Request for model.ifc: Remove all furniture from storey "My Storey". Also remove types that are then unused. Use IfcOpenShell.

First a look at what the model holds.

```python
import ifcopenshell
import ifcopenshell.util.element

model = ifcopenshell.open("model.ifc")
print(model.schema)
storey = next(s for s in model.by_type("IfcBuildingStorey") if s.Name == "My Storey")
furniture = [e for e in ifcopenshell.util.element.get_decomposition(storey) if e.is_a("IfcFurnishingElement")]
seen = {}
for e in furniture:
    element_type = ifcopenshell.util.element.get_type(e)
    name = element_type.Name if element_type not in (None, e) else None
    seen[name] = seen.get(name, 0) + 1
for name, count in sorted(seen.items(), key=str):
    print(count, "x", name)
```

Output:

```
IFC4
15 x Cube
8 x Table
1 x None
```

```python
import ifcopenshell
import ifcopenshell.api.root
import ifcopenshell.util.element

model = ifcopenshell.open("model.ifc")

storey = next(s for s in model.by_type("IfcBuildingStorey") if s.Name == "My Storey")
furniture = [e for e in ifcopenshell.util.element.get_decomposition(storey) if e.is_a("IfcFurnishingElement")]
types = {ifcopenshell.util.element.get_type(e) for e in furniture} - {None, *furniture}

for e in furniture:
    ifcopenshell.api.root.remove_product(model, product=e)
print(len(furniture), "removed")

unused = [t for t in types if not ifcopenshell.util.element.get_types(t)]
for t in unused:
    ifcopenshell.api.root.remove_product(model, product=t)
print(len(unused), "unused types removed")

model.write("model_edited.ifc")
```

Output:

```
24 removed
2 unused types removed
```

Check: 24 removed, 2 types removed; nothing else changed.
